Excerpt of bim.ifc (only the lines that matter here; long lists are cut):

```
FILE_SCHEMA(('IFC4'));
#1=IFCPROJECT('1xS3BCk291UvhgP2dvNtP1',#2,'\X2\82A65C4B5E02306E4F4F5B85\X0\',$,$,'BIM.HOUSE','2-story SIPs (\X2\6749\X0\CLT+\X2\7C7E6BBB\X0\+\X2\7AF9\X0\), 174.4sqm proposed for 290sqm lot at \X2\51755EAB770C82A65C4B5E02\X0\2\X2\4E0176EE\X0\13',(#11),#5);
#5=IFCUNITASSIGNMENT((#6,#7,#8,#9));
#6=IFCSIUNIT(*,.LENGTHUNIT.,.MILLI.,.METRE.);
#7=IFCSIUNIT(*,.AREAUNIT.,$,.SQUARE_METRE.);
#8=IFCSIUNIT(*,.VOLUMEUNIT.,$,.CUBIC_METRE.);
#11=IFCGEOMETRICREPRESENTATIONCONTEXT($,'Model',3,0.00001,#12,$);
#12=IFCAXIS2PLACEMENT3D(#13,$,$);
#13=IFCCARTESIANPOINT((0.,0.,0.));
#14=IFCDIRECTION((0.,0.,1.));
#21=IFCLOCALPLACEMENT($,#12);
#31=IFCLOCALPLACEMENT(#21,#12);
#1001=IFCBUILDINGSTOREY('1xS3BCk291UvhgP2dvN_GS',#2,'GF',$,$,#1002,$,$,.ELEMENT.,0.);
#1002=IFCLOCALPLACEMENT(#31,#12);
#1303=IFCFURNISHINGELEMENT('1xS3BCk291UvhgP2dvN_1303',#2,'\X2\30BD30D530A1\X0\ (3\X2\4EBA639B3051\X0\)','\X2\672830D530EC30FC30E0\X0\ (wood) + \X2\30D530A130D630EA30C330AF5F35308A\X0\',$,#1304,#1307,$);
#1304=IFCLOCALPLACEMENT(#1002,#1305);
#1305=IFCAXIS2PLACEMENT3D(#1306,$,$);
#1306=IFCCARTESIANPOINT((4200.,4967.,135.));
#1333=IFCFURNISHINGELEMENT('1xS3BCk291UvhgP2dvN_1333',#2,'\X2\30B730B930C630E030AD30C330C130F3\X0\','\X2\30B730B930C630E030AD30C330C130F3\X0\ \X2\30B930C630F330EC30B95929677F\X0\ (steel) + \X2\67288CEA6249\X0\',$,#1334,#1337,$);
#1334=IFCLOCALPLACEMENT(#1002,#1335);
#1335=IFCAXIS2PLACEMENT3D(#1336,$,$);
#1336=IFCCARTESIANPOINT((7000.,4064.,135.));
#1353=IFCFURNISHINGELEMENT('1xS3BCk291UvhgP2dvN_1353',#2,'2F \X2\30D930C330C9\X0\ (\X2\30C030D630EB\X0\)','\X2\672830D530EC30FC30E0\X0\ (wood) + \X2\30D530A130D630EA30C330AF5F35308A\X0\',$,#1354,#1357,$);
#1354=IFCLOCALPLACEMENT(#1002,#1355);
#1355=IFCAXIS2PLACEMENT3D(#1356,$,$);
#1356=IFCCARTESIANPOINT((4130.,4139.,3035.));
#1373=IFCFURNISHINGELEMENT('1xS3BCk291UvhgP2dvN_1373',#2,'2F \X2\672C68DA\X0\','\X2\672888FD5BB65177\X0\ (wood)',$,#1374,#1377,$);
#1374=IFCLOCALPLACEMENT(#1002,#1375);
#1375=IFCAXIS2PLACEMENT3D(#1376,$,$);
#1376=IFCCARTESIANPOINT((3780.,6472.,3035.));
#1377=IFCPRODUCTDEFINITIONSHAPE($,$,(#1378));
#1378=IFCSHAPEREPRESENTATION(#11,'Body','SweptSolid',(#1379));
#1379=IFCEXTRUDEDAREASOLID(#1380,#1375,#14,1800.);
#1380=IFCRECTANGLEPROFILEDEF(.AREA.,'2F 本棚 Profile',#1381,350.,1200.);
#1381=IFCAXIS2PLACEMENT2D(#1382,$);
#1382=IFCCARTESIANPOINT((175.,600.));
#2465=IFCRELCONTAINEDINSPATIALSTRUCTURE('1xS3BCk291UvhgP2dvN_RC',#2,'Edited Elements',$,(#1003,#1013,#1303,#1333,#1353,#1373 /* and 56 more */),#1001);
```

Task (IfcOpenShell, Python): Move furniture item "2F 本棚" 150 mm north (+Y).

```python
import ifcopenshell
import ifcopenshell.api.geometry
import ifcopenshell.util.placement
import ifcopenshell.util.unit

model = ifcopenshell.open("bim.ifc")
unit_scale = ifcopenshell.util.unit.calculate_unit_scale(model)

item = model.by_guid("1xS3BCk291UvhgP2dvN_1373")
matrix = ifcopenshell.util.placement.get_local_placement(item.ObjectPlacement)
matrix[1, 3] += 0.15 / unit_scale
ifcopenshell.api.geometry.edit_object_placement(model, product=item, matrix=matrix, is_si=False)

print(ifcopenshell.util.placement.get_local_placement(item.ObjectPlacement).round(3) + 0.0)

model.write("bim_v2.ifc")
```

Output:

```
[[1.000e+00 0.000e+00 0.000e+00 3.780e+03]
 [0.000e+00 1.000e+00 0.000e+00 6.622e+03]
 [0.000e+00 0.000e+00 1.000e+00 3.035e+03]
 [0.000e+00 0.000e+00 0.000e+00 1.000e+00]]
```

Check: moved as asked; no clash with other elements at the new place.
